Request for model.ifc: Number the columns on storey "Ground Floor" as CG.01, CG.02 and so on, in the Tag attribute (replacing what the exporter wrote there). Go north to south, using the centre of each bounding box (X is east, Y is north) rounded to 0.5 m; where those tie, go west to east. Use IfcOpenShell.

First a look at what the model holds.

```python
import ifcopenshell
import ifcopenshell.util.element
import ifcopenshell.util.placement

model = ifcopenshell.open("model.ifc")
print(model.schema)
storey = next(s for s in model.by_type("IfcBuildingStorey") if s.Name == "Ground Floor")
columns = [e for e in ifcopenshell.util.element.get_decomposition(storey) if e.is_a("IfcColumn")]
for e in sorted(columns, key=lambda e: e.id()):
    origin = ifcopenshell.util.placement.get_local_placement(e.ObjectPlacement)[:3, 3]
    print(e.id(), e.Tag, e.Name, origin.round(2) + 0.0, sep=" | ")
```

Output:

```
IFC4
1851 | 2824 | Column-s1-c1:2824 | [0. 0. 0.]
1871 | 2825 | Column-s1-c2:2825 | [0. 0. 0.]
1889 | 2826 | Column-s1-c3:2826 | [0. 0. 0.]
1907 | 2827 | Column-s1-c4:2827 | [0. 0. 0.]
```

```python
import ifcopenshell
import ifcopenshell.geom
import ifcopenshell.util.element
import ifcopenshell.util.shape

model = ifcopenshell.open("model.ifc")
settings = ifcopenshell.geom.settings()
settings.set("use-world-coords", True)


def centre(element):
    shape = ifcopenshell.geom.create_shape(settings, element)
    return ifcopenshell.util.shape.get_bbox_centroid(shape.geometry)


storey = next(s for s in model.by_type("IfcBuildingStorey") if s.Name == "Ground Floor")
columns = [e for e in ifcopenshell.util.element.get_decomposition(storey) if e.is_a("IfcColumn")]

# Insertion points can sit at a corner or the storey origin, so sort by the geometry (in metres).
centres = {e: centre(e) for e in columns}
columns.sort(key=lambda e: (-round(centres[e][1] / 0.5), centres[e][0]))

for i, e in enumerate(columns, start=1):
    number = f"CG.{i:02d}"
    e.Tag = number
    print(e.id(), number)

model.write("model_rev.ifc")
```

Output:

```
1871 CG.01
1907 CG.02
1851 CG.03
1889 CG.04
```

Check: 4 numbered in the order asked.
